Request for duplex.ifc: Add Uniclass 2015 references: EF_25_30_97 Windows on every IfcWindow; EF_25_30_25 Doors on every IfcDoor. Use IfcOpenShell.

First a look at what the model holds.

```python
import ifcopenshell

model = ifcopenshell.open("duplex.ifc")
print(model.schema)
print("classifications:", [c.Name for c in model.by_type("IfcClassification")])
for ifc_class in ("IfcDoor", "IfcRoof", "IfcStair", "IfcWall", "IfcWindow"):
    print(ifc_class, len(model.by_type(ifc_class)))
```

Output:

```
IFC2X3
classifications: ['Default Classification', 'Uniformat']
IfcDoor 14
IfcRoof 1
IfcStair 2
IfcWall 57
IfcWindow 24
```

```python
import ifcopenshell
import ifcopenshell.api.classification

model = ifcopenshell.open("duplex.ifc")

# IFC2X3 requires Source and Edition and has no link from the project to the system.
system = model.create_entity("IfcClassification", Source="NBS", Edition="2015", Name="Uniclass 2015")

codes = {
    "IfcWindow": ("EF_25_30_97", "Windows"),
    "IfcDoor": ("EF_25_30_25", "Doors"),
}
for ifc_class, (code, name) in codes.items():
    products = model.by_type(ifc_class)
    ifcopenshell.api.classification.add_reference(
        model, products=products, classification=system, identification=code, name=name
    )
    print(code, len(products))

model.write("duplex_edited.ifc")
```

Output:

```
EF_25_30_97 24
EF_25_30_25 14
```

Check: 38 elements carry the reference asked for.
